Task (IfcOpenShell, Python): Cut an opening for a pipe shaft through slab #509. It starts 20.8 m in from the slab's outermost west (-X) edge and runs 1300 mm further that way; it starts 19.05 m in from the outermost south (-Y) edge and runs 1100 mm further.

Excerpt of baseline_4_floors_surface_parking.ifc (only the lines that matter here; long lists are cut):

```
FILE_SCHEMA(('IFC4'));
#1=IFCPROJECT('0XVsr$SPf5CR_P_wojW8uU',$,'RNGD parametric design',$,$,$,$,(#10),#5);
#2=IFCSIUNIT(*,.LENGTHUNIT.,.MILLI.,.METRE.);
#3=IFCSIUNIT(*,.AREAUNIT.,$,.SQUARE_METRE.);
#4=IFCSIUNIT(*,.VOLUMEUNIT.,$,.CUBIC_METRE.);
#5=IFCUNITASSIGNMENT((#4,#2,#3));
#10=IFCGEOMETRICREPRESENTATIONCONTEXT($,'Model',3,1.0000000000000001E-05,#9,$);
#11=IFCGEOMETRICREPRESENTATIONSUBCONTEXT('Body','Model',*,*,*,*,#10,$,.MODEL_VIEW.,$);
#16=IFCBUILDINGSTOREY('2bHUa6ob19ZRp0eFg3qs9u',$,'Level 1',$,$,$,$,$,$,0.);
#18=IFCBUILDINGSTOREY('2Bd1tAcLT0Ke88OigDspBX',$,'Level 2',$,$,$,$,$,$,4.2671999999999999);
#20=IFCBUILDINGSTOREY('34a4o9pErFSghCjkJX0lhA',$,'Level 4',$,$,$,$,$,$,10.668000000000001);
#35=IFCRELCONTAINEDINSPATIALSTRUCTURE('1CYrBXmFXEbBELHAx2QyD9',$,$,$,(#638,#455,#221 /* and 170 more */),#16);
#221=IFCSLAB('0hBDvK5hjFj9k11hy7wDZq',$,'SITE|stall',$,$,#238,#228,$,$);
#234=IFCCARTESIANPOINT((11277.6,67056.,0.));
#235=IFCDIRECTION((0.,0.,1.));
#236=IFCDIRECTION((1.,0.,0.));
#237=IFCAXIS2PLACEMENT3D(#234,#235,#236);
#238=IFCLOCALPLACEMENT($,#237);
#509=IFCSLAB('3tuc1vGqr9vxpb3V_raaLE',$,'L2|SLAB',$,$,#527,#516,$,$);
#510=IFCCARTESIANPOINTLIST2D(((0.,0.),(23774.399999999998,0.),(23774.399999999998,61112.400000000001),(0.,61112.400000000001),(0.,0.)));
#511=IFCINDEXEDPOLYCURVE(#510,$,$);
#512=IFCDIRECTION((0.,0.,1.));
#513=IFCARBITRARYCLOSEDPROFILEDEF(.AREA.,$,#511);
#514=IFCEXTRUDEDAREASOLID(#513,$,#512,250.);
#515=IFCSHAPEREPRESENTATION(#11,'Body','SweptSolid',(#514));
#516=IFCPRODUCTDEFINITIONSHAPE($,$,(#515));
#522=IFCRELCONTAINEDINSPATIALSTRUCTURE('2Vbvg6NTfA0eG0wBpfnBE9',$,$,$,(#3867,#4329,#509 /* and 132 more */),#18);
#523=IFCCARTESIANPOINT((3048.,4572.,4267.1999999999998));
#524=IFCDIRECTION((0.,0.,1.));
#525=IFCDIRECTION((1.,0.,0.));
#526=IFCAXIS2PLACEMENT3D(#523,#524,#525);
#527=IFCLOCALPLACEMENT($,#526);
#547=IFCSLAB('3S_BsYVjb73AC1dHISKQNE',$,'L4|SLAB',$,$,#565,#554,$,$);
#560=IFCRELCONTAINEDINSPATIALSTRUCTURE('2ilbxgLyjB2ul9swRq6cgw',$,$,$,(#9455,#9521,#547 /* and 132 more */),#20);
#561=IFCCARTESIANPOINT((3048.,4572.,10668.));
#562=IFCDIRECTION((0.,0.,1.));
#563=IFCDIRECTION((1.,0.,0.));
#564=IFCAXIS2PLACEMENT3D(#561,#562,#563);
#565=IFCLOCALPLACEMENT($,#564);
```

```python
import numpy as np
import ifcopenshell
import ifcopenshell.api.feature
import ifcopenshell.api.geometry
import ifcopenshell.api.root
import ifcopenshell.geom
import ifcopenshell.util.placement
import ifcopenshell.util.representation
import ifcopenshell.util.shape
import ifcopenshell.util.unit

model = ifcopenshell.open("baseline_4_floors_surface_parking.ifc")
unit_scale = ifcopenshell.util.unit.calculate_unit_scale(model)
settings = ifcopenshell.geom.settings()


def volume(element):
    """Net volume in cubic metres, openings subtracted."""
    shape = ifcopenshell.geom.create_shape(settings, element)
    return ifcopenshell.util.shape.get_volume(shape.geometry)


slab = model.by_guid("3tuc1vGqr9vxpb3V_raaLE")
before = volume(slab)

# Extent in the slab's own axes, in metres. The edges named are its -X and -Y sides.
slab_shape = ifcopenshell.geom.create_shape(settings, slab)
vertices = ifcopenshell.util.shape.get_vertices(slab_shape.geometry)
x_min, y_min, bottom = vertices.min(axis=0)
top = vertices[:, 2].max()

opening = ifcopenshell.api.root.create_entity(model, ifc_class="IfcOpeningElement", name="Pipe shaft opening", predefined_type="OPENING")
context = ifcopenshell.util.representation.get_context(model, "Model", "Body", "MODEL_VIEW")
width, depth = 1.3, 1.1
outline = [(0.0, 0.0), (width, 0.0), (width, depth), (0.0, depth), (0.0, 0.0)]
# Overshoot both faces by 50 mm so the cut is clean.
shape = ifcopenshell.api.geometry.add_slab_representation(
    model, context=context, depth=top - bottom + 0.1, polyline=outline
)
ifcopenshell.api.geometry.assign_representation(model, product=opening, representation=shape)

matrix = ifcopenshell.util.placement.get_local_placement(slab.ObjectPlacement)
matrix[:, 3] = matrix @ np.append(np.array([x_min + 20.8, y_min + 19.05, bottom - 0.05]) / unit_scale, 1.0)
ifcopenshell.api.geometry.edit_object_placement(model, product=opening, matrix=matrix, is_si=False)
ifcopenshell.api.feature.add_feature(model, feature=opening, element=slab)

after = volume(slab)

print(f"slab volume {before:.3f} -> {after:.3f} m3")

model.write("baseline_4_floors_surface_parking_v2.ifc")
```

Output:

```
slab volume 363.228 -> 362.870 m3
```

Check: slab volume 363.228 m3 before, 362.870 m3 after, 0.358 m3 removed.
